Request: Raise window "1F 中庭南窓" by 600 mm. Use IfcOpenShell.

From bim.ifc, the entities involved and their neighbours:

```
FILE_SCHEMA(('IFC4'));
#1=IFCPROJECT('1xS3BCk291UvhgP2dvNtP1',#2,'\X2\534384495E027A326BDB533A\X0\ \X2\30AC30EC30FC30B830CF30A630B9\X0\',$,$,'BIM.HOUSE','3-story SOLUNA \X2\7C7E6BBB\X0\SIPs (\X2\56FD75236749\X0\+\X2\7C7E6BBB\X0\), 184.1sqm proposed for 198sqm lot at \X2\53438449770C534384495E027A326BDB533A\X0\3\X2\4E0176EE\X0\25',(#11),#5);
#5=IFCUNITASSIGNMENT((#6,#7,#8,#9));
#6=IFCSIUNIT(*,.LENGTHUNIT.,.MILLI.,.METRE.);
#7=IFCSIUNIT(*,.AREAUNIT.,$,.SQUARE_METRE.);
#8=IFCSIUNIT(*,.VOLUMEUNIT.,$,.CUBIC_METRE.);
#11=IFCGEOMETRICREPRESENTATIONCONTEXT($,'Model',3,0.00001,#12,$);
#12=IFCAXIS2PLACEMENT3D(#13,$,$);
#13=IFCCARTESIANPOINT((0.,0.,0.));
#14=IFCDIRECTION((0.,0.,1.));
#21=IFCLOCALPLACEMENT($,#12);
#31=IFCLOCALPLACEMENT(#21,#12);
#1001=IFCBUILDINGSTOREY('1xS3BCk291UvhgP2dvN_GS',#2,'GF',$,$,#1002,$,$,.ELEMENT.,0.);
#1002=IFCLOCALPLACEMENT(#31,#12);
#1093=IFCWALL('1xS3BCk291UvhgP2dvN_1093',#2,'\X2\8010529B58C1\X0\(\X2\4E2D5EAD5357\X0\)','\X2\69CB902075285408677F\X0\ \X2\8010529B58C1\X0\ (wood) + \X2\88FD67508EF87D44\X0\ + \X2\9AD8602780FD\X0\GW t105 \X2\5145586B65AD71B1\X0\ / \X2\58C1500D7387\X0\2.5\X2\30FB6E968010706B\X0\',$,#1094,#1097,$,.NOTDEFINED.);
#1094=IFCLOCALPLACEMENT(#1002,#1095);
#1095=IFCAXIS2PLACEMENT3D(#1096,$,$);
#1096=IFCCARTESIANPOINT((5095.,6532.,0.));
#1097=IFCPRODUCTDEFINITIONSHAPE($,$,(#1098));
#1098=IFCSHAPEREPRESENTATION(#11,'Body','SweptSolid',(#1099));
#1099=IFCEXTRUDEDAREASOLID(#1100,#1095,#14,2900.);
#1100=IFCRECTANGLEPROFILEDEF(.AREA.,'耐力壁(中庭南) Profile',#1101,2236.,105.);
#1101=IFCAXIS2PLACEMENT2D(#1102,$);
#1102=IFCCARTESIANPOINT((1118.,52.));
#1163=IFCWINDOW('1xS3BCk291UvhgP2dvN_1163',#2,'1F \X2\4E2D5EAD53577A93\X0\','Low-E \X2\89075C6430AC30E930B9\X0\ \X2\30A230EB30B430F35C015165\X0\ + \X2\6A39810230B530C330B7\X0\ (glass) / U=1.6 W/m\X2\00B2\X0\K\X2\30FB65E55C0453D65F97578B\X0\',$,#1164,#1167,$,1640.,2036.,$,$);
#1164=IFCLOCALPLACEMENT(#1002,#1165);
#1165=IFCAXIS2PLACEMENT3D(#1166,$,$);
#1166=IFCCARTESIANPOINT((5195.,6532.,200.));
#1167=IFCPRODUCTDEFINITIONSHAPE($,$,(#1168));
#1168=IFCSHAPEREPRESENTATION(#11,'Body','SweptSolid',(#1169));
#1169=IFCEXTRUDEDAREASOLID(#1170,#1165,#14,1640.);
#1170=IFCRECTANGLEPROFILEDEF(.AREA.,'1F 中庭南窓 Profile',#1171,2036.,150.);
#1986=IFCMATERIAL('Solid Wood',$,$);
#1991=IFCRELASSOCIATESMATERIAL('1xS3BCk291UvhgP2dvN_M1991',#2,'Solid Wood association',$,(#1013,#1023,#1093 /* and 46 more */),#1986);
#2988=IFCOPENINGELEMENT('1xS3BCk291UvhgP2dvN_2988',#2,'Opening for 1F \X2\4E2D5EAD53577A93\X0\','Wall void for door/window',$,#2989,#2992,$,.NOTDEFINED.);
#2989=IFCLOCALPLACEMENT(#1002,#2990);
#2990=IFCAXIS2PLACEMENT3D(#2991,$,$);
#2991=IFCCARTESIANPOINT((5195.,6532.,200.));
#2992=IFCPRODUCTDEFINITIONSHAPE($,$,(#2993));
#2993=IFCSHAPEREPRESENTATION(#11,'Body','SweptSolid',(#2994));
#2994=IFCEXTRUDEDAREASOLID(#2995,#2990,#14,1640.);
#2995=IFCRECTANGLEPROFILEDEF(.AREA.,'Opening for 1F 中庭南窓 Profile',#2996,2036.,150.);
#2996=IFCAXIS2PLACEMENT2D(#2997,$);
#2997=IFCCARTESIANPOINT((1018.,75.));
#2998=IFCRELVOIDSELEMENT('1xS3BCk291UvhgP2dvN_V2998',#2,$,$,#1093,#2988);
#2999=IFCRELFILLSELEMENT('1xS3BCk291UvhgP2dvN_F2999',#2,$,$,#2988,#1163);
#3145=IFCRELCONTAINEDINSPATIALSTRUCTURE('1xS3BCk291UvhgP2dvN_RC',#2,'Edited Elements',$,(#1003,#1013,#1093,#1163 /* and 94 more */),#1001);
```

```python
import numpy as np
import ifcopenshell
import ifcopenshell.api.geometry
import ifcopenshell.util.placement
import ifcopenshell.util.unit

model = ifcopenshell.open("bim.ifc")
unit_scale = ifcopenshell.util.unit.calculate_unit_scale(model)

window = model.by_id(1163)
opening = window.FillsVoids[0].RelatingOpeningElement
dz = 0.6 / unit_scale

shift = np.array([0.0, 0.0, dz])
# The window is not placed relative to its opening, so move both.
for product in (opening, window):
    matrix = ifcopenshell.util.placement.get_local_placement(product.ObjectPlacement)
    matrix[:3, 3] += shift
    ifcopenshell.api.geometry.edit_object_placement(model, product=product, matrix=matrix, is_si=False)

print(f"moved by {dz * unit_scale:+.3f} m")

model.write("bim_v2.ifc")
```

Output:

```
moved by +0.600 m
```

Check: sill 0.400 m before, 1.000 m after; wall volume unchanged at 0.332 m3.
